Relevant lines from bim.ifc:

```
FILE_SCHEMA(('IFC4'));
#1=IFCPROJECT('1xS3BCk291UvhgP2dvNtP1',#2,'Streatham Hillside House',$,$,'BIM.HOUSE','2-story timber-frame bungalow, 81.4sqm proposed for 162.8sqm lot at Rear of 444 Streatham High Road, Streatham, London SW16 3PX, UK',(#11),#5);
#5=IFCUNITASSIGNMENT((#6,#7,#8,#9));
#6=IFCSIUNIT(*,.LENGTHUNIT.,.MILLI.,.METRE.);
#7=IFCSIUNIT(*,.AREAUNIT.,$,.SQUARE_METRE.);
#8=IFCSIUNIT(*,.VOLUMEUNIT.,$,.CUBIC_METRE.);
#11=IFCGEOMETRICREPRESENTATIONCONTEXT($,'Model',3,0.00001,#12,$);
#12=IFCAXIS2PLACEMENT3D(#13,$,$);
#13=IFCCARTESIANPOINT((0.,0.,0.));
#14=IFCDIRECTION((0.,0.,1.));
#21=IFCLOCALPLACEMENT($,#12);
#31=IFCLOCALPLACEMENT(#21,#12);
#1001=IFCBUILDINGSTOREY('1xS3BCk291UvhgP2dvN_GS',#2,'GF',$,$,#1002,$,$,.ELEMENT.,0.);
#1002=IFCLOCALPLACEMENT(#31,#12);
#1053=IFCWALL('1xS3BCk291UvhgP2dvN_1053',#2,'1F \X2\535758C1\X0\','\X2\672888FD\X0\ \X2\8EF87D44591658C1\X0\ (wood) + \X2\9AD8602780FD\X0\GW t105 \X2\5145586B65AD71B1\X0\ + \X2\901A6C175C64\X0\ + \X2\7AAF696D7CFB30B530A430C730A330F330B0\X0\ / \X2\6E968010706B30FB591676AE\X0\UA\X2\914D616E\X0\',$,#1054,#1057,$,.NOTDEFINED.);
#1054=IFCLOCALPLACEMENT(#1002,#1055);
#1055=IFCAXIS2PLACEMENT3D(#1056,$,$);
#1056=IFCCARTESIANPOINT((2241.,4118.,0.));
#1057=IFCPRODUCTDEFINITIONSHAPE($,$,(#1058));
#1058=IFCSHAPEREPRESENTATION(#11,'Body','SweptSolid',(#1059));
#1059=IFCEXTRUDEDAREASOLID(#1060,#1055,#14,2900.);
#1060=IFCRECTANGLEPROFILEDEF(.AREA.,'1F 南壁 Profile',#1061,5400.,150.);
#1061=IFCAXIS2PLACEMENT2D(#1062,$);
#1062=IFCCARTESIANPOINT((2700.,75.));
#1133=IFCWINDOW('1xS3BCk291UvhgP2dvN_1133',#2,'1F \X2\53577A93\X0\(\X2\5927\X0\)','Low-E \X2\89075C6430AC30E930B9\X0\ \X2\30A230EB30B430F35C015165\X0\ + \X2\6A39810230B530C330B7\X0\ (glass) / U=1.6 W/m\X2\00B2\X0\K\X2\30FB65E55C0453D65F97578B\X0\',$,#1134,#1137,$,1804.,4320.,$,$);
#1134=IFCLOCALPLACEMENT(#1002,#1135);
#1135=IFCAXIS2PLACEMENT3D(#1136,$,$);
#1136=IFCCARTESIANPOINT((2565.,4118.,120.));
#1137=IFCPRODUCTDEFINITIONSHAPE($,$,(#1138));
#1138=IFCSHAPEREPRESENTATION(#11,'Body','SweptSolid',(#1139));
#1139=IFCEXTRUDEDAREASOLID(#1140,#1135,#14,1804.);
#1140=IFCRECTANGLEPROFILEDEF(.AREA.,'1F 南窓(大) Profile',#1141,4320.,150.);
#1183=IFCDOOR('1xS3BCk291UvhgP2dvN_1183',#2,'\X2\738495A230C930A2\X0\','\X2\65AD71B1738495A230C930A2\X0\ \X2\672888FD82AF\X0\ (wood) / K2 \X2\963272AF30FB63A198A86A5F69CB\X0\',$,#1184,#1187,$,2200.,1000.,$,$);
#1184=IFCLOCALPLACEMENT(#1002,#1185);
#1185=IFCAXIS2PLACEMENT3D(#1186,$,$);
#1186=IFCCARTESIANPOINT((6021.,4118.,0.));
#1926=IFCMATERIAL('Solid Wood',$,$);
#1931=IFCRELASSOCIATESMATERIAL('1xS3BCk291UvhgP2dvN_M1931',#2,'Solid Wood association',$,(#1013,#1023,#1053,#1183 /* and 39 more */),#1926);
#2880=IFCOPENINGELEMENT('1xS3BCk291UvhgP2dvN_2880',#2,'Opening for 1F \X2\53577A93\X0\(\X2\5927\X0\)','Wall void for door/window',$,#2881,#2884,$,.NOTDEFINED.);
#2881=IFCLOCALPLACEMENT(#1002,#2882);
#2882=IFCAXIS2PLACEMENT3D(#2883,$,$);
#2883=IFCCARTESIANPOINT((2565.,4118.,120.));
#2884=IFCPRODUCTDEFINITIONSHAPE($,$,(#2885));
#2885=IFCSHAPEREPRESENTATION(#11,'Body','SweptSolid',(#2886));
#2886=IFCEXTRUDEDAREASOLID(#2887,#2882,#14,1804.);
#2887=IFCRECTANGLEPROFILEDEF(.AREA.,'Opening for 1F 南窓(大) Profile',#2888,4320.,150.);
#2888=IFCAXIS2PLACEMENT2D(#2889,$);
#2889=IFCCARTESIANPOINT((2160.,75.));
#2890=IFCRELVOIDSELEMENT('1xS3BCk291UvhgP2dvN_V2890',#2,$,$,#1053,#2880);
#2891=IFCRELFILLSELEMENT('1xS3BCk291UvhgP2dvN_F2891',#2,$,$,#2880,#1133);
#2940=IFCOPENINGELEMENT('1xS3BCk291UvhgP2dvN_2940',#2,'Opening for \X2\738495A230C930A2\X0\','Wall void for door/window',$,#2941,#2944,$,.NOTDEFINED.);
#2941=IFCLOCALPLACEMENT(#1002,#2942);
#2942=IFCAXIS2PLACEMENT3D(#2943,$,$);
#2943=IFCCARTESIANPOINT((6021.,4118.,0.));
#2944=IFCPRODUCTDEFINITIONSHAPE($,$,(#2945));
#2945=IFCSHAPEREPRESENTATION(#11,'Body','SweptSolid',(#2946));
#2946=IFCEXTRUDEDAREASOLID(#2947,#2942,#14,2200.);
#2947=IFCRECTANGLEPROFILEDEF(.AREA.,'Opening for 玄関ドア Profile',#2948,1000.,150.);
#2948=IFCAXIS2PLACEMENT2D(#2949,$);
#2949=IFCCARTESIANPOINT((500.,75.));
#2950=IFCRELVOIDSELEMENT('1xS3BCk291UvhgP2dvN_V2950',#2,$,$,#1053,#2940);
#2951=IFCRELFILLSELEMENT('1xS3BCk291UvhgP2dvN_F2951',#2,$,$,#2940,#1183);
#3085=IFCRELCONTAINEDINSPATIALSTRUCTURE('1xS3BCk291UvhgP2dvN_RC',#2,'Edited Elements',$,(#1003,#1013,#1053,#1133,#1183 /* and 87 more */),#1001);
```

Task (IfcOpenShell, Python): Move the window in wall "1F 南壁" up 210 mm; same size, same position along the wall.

```python
import numpy as np
import ifcopenshell
import ifcopenshell.api.geometry
import ifcopenshell.util.placement
import ifcopenshell.util.unit

model = ifcopenshell.open("bim.ifc")
unit_scale = ifcopenshell.util.unit.calculate_unit_scale(model)

window = model.by_id(1133)
opening = window.FillsVoids[0].RelatingOpeningElement
dz = 0.21 / unit_scale

shift = np.array([0.0, 0.0, dz])
# The window is not placed relative to its opening, so move both.
for product in (opening, window):
    matrix = ifcopenshell.util.placement.get_local_placement(product.ObjectPlacement)
    matrix[:3, 3] += shift
    ifcopenshell.api.geometry.edit_object_placement(model, product=product, matrix=matrix, is_si=False)

print(f"moved by {dz * unit_scale:+.3f} m")

model.write("bim_v2.ifc")
```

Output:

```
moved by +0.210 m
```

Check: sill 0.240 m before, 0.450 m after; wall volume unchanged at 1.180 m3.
